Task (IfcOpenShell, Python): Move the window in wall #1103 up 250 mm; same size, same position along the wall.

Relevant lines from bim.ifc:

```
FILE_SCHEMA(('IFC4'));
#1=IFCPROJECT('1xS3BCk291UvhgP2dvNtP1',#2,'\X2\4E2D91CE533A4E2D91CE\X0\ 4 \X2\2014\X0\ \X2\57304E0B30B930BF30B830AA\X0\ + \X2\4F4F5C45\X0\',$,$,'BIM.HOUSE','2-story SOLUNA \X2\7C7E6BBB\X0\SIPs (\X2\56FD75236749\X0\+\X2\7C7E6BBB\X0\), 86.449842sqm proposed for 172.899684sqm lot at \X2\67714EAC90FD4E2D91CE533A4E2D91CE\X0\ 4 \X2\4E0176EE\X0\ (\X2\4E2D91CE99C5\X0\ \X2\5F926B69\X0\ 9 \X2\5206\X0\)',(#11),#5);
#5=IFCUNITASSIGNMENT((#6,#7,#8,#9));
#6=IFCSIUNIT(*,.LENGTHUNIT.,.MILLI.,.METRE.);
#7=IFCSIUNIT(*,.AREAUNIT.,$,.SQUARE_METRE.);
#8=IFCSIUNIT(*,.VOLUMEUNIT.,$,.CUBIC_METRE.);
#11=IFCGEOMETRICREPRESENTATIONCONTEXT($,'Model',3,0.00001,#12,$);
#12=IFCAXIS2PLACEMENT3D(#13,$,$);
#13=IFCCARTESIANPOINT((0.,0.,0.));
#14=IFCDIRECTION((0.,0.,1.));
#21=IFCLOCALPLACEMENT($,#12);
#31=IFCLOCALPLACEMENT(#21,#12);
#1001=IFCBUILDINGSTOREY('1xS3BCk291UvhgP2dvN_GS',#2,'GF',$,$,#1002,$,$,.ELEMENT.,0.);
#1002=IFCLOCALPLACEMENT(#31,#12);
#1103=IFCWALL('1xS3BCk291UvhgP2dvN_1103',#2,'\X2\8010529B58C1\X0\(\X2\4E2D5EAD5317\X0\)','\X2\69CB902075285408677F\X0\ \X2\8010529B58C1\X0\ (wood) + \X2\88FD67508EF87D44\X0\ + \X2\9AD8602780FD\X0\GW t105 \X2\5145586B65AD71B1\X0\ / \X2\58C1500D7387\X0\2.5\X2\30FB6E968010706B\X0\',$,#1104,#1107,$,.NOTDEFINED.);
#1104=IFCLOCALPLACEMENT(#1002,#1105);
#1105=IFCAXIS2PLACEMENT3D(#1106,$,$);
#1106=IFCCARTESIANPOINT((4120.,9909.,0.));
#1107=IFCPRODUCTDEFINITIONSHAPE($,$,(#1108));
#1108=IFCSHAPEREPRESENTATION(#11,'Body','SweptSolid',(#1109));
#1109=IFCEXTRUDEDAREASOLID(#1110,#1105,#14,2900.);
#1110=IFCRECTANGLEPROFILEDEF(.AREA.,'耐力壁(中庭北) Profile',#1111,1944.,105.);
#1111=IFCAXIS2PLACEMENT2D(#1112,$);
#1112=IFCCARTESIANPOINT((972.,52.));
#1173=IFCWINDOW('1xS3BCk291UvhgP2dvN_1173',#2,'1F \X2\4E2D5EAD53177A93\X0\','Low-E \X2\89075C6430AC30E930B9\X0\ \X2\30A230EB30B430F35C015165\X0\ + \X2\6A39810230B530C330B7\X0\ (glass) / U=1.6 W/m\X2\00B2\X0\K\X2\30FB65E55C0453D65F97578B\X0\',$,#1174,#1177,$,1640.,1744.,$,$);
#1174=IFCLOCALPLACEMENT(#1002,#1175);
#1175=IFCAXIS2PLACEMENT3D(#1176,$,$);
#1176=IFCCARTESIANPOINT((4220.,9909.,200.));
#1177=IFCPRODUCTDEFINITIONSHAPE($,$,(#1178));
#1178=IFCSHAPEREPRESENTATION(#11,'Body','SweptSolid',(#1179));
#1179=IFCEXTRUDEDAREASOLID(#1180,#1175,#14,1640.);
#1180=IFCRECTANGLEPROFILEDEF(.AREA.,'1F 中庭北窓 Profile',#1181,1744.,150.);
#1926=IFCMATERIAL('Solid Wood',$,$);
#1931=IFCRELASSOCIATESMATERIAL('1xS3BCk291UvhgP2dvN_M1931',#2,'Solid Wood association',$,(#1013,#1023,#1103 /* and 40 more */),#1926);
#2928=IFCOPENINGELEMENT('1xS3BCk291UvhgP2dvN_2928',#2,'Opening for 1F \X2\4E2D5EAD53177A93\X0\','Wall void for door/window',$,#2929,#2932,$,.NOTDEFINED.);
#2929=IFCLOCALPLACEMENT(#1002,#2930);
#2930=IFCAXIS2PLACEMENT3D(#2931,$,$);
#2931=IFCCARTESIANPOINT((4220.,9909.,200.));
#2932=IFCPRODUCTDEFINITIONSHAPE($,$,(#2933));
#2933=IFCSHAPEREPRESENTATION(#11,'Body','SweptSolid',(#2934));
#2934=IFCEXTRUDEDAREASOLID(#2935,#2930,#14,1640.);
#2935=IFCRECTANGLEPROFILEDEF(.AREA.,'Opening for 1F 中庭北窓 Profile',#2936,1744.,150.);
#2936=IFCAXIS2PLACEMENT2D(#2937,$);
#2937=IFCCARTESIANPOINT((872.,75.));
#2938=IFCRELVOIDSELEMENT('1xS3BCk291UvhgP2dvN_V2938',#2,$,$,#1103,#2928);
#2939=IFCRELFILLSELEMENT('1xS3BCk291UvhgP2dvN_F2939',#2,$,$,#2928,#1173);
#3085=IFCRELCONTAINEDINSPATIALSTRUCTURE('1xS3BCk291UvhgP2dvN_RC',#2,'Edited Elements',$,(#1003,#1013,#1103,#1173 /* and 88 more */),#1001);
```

```python
import numpy as np
import ifcopenshell
import ifcopenshell.api.geometry
import ifcopenshell.util.placement
import ifcopenshell.util.unit

model = ifcopenshell.open("bim.ifc")
unit_scale = ifcopenshell.util.unit.calculate_unit_scale(model)

window = model.by_guid("1xS3BCk291UvhgP2dvN_1173")
opening = window.FillsVoids[0].RelatingOpeningElement
dz = 0.25 / unit_scale

shift = np.array([0.0, 0.0, dz])
# The window is not placed relative to its opening, so move both.
for product in (opening, window):
    matrix = ifcopenshell.util.placement.get_local_placement(product.ObjectPlacement)
    matrix[:3, 3] += shift
    ifcopenshell.api.geometry.edit_object_placement(model, product=product, matrix=matrix, is_si=False)

print(f"moved by {dz * unit_scale:+.3f} m")

model.write("bim_updated.ifc")
```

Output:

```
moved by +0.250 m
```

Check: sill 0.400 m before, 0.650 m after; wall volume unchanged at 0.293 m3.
